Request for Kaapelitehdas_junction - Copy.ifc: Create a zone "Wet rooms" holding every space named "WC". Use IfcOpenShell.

First a look at what the model holds.

```python
import ifcopenshell

model = ifcopenshell.open("Kaapelitehdas_junction - Copy.ifc")
print(model.schema)
seen = {}
for space in model.by_type("IfcSpace"):
    seen[space.LongName] = seen.get(space.LongName, 0) + 1
for name, count in sorted(seen.items(), key=str):
    print(count, "x", name)
print("zones:", [z.Name for z in model.by_type("IfcZone")][:20])
```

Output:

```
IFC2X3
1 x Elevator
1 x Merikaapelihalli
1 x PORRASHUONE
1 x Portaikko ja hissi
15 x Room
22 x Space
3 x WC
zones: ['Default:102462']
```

```python
import ifcopenshell
import ifcopenshell.api.group
import ifcopenshell.api.root

model = ifcopenshell.open("Kaapelitehdas_junction - Copy.ifc")

names = {"WC"}
spaces = [s for s in model.by_type("IfcSpace") if s.LongName in names]

zone = ifcopenshell.api.root.create_entity(model, ifc_class="IfcZone", name="Wet rooms")
ifcopenshell.api.group.assign_group(model, products=spaces, group=zone)
print(len(spaces), "spaces in", zone.Name)

model.write("Kaapelitehdas_junction - Copy_v2.ifc")
```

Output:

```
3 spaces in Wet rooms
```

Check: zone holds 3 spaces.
